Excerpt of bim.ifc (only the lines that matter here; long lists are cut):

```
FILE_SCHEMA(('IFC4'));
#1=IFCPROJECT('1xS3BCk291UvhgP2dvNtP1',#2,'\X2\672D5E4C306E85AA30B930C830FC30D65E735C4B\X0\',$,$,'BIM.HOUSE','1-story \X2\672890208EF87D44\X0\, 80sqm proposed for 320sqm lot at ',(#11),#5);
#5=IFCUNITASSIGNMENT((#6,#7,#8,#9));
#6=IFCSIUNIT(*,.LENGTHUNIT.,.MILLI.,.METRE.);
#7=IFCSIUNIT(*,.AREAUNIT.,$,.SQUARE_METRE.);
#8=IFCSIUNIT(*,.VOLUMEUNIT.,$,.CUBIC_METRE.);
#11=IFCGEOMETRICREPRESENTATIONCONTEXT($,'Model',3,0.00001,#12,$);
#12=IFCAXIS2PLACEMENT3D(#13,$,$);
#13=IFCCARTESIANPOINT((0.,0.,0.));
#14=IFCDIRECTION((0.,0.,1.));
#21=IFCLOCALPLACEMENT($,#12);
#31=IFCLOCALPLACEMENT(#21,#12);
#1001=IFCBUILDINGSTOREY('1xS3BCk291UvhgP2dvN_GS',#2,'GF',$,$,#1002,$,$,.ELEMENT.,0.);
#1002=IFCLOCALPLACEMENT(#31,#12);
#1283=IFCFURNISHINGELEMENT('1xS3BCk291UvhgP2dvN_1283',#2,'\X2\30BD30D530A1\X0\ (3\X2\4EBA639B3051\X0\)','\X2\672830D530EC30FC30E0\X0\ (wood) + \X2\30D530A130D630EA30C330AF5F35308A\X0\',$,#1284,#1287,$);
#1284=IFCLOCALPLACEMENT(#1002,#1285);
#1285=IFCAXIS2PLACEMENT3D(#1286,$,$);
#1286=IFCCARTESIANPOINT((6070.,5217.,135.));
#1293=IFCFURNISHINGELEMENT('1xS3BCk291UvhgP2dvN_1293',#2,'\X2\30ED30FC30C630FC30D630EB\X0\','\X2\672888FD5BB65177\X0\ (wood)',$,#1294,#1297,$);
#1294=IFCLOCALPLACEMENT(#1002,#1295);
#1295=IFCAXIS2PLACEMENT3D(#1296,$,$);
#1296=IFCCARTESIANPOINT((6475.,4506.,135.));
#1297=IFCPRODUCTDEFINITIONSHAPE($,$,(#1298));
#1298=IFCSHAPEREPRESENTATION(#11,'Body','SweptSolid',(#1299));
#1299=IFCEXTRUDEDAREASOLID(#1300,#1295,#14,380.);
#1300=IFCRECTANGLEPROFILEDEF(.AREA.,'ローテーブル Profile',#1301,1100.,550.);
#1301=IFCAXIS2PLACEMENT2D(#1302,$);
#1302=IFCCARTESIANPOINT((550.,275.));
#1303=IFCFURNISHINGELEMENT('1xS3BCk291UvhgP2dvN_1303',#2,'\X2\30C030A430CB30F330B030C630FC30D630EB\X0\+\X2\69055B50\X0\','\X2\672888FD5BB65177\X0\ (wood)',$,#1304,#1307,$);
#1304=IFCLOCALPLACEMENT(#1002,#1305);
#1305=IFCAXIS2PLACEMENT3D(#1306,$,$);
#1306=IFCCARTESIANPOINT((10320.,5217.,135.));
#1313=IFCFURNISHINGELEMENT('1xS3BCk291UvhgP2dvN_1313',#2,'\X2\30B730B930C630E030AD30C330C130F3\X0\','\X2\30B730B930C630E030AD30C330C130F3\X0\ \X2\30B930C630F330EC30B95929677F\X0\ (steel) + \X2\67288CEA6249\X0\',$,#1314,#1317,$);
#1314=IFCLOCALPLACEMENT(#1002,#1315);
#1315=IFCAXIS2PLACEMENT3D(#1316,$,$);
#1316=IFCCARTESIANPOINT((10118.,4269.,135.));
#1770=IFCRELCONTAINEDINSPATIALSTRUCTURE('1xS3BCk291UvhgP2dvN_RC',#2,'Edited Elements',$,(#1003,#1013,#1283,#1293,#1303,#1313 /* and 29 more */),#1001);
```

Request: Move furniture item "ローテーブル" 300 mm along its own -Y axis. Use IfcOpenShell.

```python
import ifcopenshell
import ifcopenshell.api.geometry
import ifcopenshell.util.placement
import ifcopenshell.util.unit

model = ifcopenshell.open("bim.ifc")
unit_scale = ifcopenshell.util.unit.calculate_unit_scale(model)

item = model.by_guid("1xS3BCk291UvhgP2dvN_1293")
matrix = ifcopenshell.util.placement.get_local_placement(item.ObjectPlacement)
matrix[:3, 3] -= matrix[:3, 1] * 0.3 / unit_scale
ifcopenshell.api.geometry.edit_object_placement(model, product=item, matrix=matrix, is_si=False)

print(ifcopenshell.util.placement.get_local_placement(item.ObjectPlacement).round(3) + 0.0)

model.write("bim_v2.ifc")
```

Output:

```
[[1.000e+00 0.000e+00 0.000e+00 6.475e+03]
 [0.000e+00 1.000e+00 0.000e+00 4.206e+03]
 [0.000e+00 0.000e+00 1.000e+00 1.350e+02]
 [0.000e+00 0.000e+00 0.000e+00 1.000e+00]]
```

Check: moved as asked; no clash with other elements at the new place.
